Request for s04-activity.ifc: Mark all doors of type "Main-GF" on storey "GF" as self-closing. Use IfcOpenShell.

First a look at what the model holds.

```python
import ifcopenshell
import ifcopenshell.util.element

model = ifcopenshell.open("s04-activity.ifc")
print(model.schema)
storey = next(s for s in model.by_type("IfcBuildingStorey") if s.Name == "GF")
doors = [e for e in ifcopenshell.util.element.get_decomposition(storey) if e.is_a("IfcDoor")]
seen = {}
for e in doors:
    element_type = ifcopenshell.util.element.get_type(e)
    key = (element_type.Name if element_type != e and element_type else None, ifcopenshell.util.element.get_pset(e, "Pset_DoorCommon", "SelfClosing"))
    seen[key] = seen.get(key, 0) + 1
for (name, value), count in sorted(seen.items(), key=str):
    print(count, "x", name, "|", value)
```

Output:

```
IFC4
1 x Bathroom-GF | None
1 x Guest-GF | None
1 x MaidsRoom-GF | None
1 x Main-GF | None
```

```python
import ifcopenshell
import ifcopenshell.api.pset
import ifcopenshell.util.element

model = ifcopenshell.open("s04-activity.ifc")

storey = next(s for s in model.by_type("IfcBuildingStorey") if s.Name == "GF")
doors = [e for e in ifcopenshell.util.element.get_decomposition(storey) if e.is_a("IfcDoor")]

count = 0
for e in doors:
    element_type = ifcopenshell.util.element.get_type(e)
    if element_type in (None, e) or element_type.Name != "Main-GF":
        continue
    # add_pset returns the element's existing set when there is one.
    pset = ifcopenshell.api.pset.add_pset(model, product=e, name="Pset_DoorCommon")
    ifcopenshell.api.pset.edit_pset(model, pset=pset, properties={"SelfClosing": True})
    count += 1

print(count, "doors updated")

model.write("s04-activity_rev.ifc")
```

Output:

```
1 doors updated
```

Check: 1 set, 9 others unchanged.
